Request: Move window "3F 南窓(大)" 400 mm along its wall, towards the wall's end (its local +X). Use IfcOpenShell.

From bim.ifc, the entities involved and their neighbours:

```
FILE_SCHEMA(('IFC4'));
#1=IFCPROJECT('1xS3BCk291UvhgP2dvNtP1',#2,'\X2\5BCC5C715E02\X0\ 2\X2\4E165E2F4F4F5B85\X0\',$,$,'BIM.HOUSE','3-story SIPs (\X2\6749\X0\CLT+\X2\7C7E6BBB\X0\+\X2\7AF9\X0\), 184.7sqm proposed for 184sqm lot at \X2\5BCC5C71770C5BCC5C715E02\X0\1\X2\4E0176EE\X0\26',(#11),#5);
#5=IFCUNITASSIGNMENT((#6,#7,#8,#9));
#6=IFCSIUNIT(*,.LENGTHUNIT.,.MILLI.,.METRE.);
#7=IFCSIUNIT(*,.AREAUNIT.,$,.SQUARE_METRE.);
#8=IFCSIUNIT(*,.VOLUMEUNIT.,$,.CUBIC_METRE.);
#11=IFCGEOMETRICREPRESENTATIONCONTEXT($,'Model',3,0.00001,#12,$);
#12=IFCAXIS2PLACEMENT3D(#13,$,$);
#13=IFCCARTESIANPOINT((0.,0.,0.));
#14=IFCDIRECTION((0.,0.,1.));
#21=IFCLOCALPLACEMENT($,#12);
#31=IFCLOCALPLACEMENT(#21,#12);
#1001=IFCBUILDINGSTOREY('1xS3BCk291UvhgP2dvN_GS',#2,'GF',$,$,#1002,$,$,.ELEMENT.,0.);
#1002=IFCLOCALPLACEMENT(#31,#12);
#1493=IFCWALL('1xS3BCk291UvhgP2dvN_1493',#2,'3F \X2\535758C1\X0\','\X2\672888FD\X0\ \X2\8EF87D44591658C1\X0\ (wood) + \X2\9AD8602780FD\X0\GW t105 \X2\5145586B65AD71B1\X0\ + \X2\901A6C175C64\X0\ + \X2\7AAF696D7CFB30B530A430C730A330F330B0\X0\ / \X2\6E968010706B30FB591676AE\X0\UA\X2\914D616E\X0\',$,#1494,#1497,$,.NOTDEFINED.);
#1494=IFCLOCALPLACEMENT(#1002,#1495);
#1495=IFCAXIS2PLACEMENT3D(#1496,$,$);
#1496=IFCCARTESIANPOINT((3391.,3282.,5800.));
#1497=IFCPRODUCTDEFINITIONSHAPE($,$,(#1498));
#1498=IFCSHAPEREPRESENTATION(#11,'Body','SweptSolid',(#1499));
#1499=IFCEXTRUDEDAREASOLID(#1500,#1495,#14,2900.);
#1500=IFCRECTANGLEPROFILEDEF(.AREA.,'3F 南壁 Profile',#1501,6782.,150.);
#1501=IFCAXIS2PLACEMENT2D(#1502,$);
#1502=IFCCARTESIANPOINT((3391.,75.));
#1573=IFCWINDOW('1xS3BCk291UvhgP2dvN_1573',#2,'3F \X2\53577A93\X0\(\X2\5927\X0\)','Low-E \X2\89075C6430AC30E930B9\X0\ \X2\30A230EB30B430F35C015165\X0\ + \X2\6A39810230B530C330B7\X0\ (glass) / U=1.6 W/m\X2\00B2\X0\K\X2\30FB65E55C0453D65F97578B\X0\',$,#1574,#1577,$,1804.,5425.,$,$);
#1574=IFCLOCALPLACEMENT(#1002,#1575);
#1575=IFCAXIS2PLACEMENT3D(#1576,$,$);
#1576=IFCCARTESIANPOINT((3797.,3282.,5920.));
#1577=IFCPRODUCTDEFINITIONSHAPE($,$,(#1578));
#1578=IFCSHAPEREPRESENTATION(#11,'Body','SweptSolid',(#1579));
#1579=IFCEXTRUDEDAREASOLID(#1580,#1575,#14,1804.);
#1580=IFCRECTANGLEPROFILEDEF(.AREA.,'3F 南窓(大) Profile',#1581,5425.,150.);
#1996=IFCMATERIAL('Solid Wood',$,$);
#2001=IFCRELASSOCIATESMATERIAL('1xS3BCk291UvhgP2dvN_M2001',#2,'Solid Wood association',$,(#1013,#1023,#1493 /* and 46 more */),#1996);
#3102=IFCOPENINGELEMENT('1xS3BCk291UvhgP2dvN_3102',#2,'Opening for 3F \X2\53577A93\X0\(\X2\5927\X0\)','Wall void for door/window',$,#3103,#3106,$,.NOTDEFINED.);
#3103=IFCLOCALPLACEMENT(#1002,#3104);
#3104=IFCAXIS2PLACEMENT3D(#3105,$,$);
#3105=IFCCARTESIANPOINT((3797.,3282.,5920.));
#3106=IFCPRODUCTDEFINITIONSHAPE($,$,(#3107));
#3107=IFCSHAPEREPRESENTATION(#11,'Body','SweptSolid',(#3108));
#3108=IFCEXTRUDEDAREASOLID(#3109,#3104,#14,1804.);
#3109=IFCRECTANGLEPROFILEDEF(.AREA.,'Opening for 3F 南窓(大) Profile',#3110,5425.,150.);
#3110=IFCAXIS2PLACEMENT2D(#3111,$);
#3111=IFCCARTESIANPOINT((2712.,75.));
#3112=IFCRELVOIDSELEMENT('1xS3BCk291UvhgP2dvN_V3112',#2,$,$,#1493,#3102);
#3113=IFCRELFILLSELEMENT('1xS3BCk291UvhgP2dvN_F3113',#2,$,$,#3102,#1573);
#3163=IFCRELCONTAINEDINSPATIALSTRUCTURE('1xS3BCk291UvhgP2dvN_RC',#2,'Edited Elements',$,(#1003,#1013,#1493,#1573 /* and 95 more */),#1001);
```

```python
import ifcopenshell
import ifcopenshell.api.geometry
import ifcopenshell.util.placement
import ifcopenshell.util.unit

model = ifcopenshell.open("bim.ifc")
unit_scale = ifcopenshell.util.unit.calculate_unit_scale(model)

window = model.by_guid("1xS3BCk291UvhgP2dvN_1573")
opening = window.FillsVoids[0].RelatingOpeningElement
wall = opening.VoidsElements[0].RelatingBuildingElement

wall_matrix = ifcopenshell.util.placement.get_local_placement(wall.ObjectPlacement)
shift = wall_matrix[:3, 0] * 0.4 / unit_scale
before = ifcopenshell.util.placement.get_local_placement(window.ObjectPlacement)[:3, 3].copy()

# The window is not placed relative to its opening, so move both.
for product in (opening, window):
    matrix = ifcopenshell.util.placement.get_local_placement(product.ObjectPlacement)
    matrix[:3, 3] += shift
    ifcopenshell.api.geometry.edit_object_placement(model, product=product, matrix=matrix, is_si=False)

after = ifcopenshell.util.placement.get_local_placement(window.ObjectPlacement)[:3, 3]
print("window moved by", (after - before).round(3) + 0.0)

model.write("bim_edited.ifc")
```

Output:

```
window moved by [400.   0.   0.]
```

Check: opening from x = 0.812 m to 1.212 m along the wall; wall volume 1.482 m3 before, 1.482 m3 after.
